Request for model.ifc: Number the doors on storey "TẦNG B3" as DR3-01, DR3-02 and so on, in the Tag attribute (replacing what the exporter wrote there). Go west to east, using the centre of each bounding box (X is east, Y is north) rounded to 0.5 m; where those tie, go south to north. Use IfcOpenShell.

First a look at what the model holds.

```python
import ifcopenshell
import ifcopenshell.util.element
import ifcopenshell.util.placement

model = ifcopenshell.open("model.ifc")
print(model.schema)
storey = next(s for s in model.by_type("IfcBuildingStorey") if s.Name == "TẦNG B3")
doors = [e for e in ifcopenshell.util.element.get_decomposition(storey) if e.is_a("IfcDoor")]
for e in sorted(doors, key=lambda e: e.id()):
    origin = ifcopenshell.util.placement.get_local_placement(e.ObjectPlacement)[:3, 3]
    print(e.id(), e.Tag, e.Name, origin.round(2) + 0.0, sep=" | ")
```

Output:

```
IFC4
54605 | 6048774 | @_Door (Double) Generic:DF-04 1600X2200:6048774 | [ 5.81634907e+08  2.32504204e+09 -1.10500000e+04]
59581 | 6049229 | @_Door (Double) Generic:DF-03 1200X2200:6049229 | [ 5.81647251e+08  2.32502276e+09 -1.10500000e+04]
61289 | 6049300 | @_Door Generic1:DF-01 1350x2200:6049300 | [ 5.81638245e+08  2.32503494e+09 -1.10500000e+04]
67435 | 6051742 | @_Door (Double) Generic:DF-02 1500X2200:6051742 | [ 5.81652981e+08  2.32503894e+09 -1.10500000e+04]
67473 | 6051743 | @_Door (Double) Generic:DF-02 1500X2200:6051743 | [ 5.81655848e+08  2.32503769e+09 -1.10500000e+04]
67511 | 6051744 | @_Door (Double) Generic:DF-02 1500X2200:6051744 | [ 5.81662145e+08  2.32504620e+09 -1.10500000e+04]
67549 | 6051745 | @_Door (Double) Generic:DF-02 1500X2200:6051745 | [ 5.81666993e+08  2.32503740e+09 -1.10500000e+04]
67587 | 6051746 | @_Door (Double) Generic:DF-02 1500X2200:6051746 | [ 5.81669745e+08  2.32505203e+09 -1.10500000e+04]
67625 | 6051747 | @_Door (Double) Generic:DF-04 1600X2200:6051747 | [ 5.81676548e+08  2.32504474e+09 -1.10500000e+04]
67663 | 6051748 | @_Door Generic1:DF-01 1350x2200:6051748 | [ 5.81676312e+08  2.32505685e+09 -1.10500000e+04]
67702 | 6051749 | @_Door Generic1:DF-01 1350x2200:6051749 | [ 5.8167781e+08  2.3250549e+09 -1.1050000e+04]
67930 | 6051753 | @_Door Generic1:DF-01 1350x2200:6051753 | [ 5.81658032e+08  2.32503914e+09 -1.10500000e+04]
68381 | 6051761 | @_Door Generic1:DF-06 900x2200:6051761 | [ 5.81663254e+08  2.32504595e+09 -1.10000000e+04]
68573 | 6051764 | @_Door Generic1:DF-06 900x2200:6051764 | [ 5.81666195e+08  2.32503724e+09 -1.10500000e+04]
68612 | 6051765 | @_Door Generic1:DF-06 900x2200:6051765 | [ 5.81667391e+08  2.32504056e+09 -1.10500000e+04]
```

```python
import ifcopenshell
import ifcopenshell.geom
import ifcopenshell.util.element
import ifcopenshell.util.shape

model = ifcopenshell.open("model.ifc")
settings = ifcopenshell.geom.settings()
settings.set("use-world-coords", True)


def centre(element):
    shape = ifcopenshell.geom.create_shape(settings, element)
    return ifcopenshell.util.shape.get_bbox_centroid(shape.geometry)


storey = next(s for s in model.by_type("IfcBuildingStorey") if s.Name == "TẦNG B3")
doors = [e for e in ifcopenshell.util.element.get_decomposition(storey) if e.is_a("IfcDoor")]

# Insertion points can sit at a corner or the storey origin, so sort by the geometry (in metres).
centres = {e: centre(e) for e in doors}
doors.sort(key=lambda e: (round(centres[e][0] / 0.5), centres[e][1]))

for i, e in enumerate(doors, start=1):
    number = f"DR3-{i:02d}"
    e.Tag = number
    print(e.id(), number)

model.write("model_v2.ifc")
```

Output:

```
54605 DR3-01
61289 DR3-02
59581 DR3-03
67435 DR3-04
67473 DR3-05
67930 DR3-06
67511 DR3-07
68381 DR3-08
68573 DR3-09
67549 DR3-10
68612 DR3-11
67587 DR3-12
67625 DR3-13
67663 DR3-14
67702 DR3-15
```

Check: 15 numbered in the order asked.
